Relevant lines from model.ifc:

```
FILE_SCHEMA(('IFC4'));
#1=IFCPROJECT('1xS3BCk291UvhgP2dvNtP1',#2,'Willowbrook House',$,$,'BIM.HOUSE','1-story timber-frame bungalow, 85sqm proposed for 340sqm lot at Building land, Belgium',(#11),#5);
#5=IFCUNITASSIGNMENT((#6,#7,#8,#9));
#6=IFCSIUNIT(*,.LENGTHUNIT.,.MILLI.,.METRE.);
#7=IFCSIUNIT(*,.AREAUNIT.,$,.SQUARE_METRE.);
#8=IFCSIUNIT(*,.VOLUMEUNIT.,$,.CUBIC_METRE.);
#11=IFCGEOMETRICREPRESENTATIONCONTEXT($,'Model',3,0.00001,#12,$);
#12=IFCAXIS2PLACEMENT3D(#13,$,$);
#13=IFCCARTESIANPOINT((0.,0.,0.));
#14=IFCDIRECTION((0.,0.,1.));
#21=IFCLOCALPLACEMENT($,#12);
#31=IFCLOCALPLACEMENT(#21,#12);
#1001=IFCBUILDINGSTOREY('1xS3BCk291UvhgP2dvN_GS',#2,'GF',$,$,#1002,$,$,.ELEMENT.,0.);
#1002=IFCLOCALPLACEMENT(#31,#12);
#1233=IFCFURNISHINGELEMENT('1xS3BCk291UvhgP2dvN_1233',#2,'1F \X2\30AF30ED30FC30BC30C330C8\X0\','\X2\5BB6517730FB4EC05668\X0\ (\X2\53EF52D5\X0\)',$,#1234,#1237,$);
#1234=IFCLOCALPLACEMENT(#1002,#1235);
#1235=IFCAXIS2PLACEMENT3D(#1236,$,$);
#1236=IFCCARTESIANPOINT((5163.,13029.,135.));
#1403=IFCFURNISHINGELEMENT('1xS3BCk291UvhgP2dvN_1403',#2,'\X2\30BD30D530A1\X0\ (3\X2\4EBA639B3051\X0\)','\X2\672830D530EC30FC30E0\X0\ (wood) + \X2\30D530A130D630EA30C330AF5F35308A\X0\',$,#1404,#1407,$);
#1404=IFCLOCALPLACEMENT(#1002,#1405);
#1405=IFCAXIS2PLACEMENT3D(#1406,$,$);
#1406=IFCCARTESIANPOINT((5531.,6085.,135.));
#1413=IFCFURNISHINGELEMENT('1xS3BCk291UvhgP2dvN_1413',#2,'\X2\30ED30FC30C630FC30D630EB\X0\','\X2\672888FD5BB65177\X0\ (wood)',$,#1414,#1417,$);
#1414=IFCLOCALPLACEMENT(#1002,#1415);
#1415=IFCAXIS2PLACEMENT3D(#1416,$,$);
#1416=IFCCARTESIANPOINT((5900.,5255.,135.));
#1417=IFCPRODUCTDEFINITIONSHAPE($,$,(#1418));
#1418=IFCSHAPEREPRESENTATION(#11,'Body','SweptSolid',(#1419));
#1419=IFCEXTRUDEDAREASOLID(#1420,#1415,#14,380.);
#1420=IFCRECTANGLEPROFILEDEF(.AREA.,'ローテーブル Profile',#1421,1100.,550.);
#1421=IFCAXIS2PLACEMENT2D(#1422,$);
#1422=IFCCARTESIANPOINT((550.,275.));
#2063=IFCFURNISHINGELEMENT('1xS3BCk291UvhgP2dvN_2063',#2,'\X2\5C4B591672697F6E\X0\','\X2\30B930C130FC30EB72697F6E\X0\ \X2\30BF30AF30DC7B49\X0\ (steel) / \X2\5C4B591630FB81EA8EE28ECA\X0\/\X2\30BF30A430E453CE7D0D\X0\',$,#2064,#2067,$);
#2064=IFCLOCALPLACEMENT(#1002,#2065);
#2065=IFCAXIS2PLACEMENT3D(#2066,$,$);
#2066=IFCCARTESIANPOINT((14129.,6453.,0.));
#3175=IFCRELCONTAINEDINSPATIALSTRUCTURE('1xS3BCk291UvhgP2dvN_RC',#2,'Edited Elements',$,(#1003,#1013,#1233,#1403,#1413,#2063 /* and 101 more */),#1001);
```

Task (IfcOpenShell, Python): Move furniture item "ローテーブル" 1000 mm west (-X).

```python
import ifcopenshell
import ifcopenshell.api.geometry
import ifcopenshell.util.placement

model = ifcopenshell.open("model.ifc")

item = model.by_guid("1xS3BCk291UvhgP2dvN_1413")
matrix = ifcopenshell.util.placement.get_local_placement(item.ObjectPlacement)
matrix[0, 3] -= 1000.0
ifcopenshell.api.geometry.edit_object_placement(model, product=item, matrix=matrix, is_si=False)

print(ifcopenshell.util.placement.get_local_placement(item.ObjectPlacement).round(3) + 0.0)

model.write("model_rev.ifc")
```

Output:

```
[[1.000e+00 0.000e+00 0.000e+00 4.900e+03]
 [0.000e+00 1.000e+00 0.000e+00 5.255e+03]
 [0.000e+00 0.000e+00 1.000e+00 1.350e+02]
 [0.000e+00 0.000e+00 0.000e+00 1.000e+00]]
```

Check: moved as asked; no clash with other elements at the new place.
